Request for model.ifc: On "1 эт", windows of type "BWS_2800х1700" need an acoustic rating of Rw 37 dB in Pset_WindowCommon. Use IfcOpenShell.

First a look at what the model holds.

```python
import ifcopenshell
import ifcopenshell.util.element

model = ifcopenshell.open("model.ifc")
print(model.schema)
storey = next(s for s in model.by_type("IfcBuildingStorey") if s.Name == "1 эт")
windows = [e for e in ifcopenshell.util.element.get_decomposition(storey) if e.is_a("IfcWindow")]
seen = {}
for e in windows:
    element_type = ifcopenshell.util.element.get_type(e)
    key = (element_type.Name if element_type != e and element_type else None, ifcopenshell.util.element.get_pset(e, "Pset_WindowCommon", "AcousticRating"))
    seen[key] = seen.get(key, 0) + 1
for (name, value), count in sorted(seen.items(), key=str):
    print(count, "x", name, "|", value)
```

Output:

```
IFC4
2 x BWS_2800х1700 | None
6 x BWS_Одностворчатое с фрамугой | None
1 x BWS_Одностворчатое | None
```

```python
import ifcopenshell
import ifcopenshell.api.pset
import ifcopenshell.util.element

model = ifcopenshell.open("model.ifc")

storey = next(s for s in model.by_type("IfcBuildingStorey") if s.Name == "1 эт")
windows = [e for e in ifcopenshell.util.element.get_decomposition(storey) if e.is_a("IfcWindow")]

count = 0
for e in windows:
    element_type = ifcopenshell.util.element.get_type(e)
    if element_type in (None, e) or element_type.Name != "BWS_2800х1700":
        continue
    # add_pset returns the element's existing set when there is one.
    pset = ifcopenshell.api.pset.add_pset(model, product=e, name="Pset_WindowCommon")
    ifcopenshell.api.pset.edit_pset(model, pset=pset, properties={"AcousticRating": "Rw 37 dB"})
    count += 1

print(count, "windows updated")

model.write("model_v2.ifc")
```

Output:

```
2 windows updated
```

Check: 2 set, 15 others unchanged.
